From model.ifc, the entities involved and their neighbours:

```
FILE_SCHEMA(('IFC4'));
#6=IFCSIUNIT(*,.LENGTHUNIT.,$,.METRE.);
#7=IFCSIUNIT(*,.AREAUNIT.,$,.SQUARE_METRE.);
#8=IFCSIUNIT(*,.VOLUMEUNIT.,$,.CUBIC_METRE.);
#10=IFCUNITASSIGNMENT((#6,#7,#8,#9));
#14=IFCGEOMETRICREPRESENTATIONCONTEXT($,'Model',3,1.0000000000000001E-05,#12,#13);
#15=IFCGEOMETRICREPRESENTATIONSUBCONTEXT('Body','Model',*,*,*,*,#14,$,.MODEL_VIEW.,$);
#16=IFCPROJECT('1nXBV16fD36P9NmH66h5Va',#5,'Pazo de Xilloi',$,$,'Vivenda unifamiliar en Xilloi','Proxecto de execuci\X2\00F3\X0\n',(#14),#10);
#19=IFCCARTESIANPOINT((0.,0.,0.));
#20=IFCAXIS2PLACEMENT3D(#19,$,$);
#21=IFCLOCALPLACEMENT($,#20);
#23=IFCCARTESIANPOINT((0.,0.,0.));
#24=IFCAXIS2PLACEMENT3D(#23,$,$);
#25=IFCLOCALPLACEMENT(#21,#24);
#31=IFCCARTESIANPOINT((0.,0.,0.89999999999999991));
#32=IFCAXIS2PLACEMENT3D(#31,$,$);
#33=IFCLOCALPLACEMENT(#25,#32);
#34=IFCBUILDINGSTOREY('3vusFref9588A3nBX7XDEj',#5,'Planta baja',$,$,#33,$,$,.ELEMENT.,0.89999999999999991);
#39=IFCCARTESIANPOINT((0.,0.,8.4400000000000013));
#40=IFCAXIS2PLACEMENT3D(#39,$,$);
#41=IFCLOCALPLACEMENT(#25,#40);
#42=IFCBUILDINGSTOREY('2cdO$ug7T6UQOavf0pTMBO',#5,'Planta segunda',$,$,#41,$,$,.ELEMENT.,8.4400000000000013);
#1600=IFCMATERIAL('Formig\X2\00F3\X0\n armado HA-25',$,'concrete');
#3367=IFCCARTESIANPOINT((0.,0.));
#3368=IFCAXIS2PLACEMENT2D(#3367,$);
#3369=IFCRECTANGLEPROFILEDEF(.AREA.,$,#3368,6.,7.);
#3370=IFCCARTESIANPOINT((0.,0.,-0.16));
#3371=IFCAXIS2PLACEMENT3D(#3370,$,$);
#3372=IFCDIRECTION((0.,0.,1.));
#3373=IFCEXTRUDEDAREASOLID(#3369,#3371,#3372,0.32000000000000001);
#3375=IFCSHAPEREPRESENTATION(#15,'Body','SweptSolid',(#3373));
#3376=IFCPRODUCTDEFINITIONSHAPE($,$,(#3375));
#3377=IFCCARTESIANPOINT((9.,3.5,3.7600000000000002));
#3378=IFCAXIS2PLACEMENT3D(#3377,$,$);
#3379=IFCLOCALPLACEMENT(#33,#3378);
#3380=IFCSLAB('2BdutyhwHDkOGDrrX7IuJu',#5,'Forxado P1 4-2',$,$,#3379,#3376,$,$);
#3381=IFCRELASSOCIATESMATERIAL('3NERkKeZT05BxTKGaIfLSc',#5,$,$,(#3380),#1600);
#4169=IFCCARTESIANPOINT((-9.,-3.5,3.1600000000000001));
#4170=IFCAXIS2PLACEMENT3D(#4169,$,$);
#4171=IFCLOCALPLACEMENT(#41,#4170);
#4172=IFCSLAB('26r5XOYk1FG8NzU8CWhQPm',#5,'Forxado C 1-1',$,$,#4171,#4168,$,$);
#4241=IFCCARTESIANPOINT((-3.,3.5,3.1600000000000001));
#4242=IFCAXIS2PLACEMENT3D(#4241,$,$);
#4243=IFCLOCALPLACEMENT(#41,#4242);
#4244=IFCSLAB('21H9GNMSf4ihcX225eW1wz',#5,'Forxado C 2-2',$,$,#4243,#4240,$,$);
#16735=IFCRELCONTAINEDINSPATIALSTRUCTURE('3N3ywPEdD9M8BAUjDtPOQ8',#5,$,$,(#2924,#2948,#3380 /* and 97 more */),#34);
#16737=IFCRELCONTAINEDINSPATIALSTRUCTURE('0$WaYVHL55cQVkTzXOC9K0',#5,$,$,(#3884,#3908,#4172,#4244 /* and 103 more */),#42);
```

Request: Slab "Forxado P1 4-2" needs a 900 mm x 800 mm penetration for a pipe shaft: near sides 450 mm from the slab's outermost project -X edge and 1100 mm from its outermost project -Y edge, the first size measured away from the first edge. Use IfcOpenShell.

```python
import numpy as np
import ifcopenshell
import ifcopenshell.api.feature
import ifcopenshell.api.geometry
import ifcopenshell.api.root
import ifcopenshell.geom
import ifcopenshell.util.placement
import ifcopenshell.util.representation
import ifcopenshell.util.shape
import ifcopenshell.util.unit

model = ifcopenshell.open("model.ifc")
unit_scale = ifcopenshell.util.unit.calculate_unit_scale(model)
settings = ifcopenshell.geom.settings()


def volume(element):
    """Net volume in cubic metres, openings subtracted."""
    shape = ifcopenshell.geom.create_shape(settings, element)
    return ifcopenshell.util.shape.get_volume(shape.geometry)


slab = model.by_guid("2BdutyhwHDkOGDrrX7IuJu")
before = volume(slab)

# Extent in the slab's own axes, in metres. The edges named are its -X and -Y sides.
slab_shape = ifcopenshell.geom.create_shape(settings, slab)
vertices = ifcopenshell.util.shape.get_vertices(slab_shape.geometry)
x_min, y_min, bottom = vertices.min(axis=0)
top = vertices[:, 2].max()

opening = ifcopenshell.api.root.create_entity(model, ifc_class="IfcOpeningElement", name="Pipe shaft opening", predefined_type="OPENING")
context = ifcopenshell.util.representation.get_context(model, "Model", "Body", "MODEL_VIEW")
width, depth = 0.9, 0.8
outline = [(0.0, 0.0), (width, 0.0), (width, depth), (0.0, depth), (0.0, 0.0)]
# Overshoot both faces by 50 mm so the cut is clean.
shape = ifcopenshell.api.geometry.add_slab_representation(
    model, context=context, depth=top - bottom + 0.1, polyline=outline
)
ifcopenshell.api.geometry.assign_representation(model, product=opening, representation=shape)

matrix = ifcopenshell.util.placement.get_local_placement(slab.ObjectPlacement)
matrix[:, 3] = matrix @ np.append(np.array([x_min + 0.45, y_min + 1.1, bottom - 0.05]) / unit_scale, 1.0)
ifcopenshell.api.geometry.edit_object_placement(model, product=opening, matrix=matrix, is_si=False)
ifcopenshell.api.feature.add_feature(model, feature=opening, element=slab)

after = volume(slab)

print(f"slab volume {before:.3f} -> {after:.3f} m3")

model.write("model_edited.ifc")
```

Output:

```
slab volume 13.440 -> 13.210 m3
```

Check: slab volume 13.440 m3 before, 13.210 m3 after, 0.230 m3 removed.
